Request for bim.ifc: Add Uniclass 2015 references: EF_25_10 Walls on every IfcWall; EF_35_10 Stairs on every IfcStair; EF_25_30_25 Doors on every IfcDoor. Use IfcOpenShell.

First a look at what the model holds.

```python
import ifcopenshell

model = ifcopenshell.open("bim.ifc")
print(model.schema)
print("classifications:", [c.Name for c in model.by_type("IfcClassification")])
for ifc_class in ("IfcDoor", "IfcRoof", "IfcStair", "IfcWall", "IfcWindow"):
    print(ifc_class, len(model.by_type(ifc_class)))
```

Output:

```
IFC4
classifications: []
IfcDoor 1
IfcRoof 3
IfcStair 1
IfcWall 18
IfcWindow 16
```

```python
import ifcopenshell
import ifcopenshell.api.classification

model = ifcopenshell.open("bim.ifc")

system = ifcopenshell.api.classification.add_classification(model, classification="Uniclass 2015")

codes = {
    "IfcWall": ("EF_25_10", "Walls"),
    "IfcStair": ("EF_35_10", "Stairs"),
    "IfcDoor": ("EF_25_30_25", "Doors"),
}
for ifc_class, (code, name) in codes.items():
    products = model.by_type(ifc_class)
    ifcopenshell.api.classification.add_reference(
        model, products=products, classification=system, identification=code, name=name
    )
    print(code, len(products))

model.write("bim-out.ifc")
```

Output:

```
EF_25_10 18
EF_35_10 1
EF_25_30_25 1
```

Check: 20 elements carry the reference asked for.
